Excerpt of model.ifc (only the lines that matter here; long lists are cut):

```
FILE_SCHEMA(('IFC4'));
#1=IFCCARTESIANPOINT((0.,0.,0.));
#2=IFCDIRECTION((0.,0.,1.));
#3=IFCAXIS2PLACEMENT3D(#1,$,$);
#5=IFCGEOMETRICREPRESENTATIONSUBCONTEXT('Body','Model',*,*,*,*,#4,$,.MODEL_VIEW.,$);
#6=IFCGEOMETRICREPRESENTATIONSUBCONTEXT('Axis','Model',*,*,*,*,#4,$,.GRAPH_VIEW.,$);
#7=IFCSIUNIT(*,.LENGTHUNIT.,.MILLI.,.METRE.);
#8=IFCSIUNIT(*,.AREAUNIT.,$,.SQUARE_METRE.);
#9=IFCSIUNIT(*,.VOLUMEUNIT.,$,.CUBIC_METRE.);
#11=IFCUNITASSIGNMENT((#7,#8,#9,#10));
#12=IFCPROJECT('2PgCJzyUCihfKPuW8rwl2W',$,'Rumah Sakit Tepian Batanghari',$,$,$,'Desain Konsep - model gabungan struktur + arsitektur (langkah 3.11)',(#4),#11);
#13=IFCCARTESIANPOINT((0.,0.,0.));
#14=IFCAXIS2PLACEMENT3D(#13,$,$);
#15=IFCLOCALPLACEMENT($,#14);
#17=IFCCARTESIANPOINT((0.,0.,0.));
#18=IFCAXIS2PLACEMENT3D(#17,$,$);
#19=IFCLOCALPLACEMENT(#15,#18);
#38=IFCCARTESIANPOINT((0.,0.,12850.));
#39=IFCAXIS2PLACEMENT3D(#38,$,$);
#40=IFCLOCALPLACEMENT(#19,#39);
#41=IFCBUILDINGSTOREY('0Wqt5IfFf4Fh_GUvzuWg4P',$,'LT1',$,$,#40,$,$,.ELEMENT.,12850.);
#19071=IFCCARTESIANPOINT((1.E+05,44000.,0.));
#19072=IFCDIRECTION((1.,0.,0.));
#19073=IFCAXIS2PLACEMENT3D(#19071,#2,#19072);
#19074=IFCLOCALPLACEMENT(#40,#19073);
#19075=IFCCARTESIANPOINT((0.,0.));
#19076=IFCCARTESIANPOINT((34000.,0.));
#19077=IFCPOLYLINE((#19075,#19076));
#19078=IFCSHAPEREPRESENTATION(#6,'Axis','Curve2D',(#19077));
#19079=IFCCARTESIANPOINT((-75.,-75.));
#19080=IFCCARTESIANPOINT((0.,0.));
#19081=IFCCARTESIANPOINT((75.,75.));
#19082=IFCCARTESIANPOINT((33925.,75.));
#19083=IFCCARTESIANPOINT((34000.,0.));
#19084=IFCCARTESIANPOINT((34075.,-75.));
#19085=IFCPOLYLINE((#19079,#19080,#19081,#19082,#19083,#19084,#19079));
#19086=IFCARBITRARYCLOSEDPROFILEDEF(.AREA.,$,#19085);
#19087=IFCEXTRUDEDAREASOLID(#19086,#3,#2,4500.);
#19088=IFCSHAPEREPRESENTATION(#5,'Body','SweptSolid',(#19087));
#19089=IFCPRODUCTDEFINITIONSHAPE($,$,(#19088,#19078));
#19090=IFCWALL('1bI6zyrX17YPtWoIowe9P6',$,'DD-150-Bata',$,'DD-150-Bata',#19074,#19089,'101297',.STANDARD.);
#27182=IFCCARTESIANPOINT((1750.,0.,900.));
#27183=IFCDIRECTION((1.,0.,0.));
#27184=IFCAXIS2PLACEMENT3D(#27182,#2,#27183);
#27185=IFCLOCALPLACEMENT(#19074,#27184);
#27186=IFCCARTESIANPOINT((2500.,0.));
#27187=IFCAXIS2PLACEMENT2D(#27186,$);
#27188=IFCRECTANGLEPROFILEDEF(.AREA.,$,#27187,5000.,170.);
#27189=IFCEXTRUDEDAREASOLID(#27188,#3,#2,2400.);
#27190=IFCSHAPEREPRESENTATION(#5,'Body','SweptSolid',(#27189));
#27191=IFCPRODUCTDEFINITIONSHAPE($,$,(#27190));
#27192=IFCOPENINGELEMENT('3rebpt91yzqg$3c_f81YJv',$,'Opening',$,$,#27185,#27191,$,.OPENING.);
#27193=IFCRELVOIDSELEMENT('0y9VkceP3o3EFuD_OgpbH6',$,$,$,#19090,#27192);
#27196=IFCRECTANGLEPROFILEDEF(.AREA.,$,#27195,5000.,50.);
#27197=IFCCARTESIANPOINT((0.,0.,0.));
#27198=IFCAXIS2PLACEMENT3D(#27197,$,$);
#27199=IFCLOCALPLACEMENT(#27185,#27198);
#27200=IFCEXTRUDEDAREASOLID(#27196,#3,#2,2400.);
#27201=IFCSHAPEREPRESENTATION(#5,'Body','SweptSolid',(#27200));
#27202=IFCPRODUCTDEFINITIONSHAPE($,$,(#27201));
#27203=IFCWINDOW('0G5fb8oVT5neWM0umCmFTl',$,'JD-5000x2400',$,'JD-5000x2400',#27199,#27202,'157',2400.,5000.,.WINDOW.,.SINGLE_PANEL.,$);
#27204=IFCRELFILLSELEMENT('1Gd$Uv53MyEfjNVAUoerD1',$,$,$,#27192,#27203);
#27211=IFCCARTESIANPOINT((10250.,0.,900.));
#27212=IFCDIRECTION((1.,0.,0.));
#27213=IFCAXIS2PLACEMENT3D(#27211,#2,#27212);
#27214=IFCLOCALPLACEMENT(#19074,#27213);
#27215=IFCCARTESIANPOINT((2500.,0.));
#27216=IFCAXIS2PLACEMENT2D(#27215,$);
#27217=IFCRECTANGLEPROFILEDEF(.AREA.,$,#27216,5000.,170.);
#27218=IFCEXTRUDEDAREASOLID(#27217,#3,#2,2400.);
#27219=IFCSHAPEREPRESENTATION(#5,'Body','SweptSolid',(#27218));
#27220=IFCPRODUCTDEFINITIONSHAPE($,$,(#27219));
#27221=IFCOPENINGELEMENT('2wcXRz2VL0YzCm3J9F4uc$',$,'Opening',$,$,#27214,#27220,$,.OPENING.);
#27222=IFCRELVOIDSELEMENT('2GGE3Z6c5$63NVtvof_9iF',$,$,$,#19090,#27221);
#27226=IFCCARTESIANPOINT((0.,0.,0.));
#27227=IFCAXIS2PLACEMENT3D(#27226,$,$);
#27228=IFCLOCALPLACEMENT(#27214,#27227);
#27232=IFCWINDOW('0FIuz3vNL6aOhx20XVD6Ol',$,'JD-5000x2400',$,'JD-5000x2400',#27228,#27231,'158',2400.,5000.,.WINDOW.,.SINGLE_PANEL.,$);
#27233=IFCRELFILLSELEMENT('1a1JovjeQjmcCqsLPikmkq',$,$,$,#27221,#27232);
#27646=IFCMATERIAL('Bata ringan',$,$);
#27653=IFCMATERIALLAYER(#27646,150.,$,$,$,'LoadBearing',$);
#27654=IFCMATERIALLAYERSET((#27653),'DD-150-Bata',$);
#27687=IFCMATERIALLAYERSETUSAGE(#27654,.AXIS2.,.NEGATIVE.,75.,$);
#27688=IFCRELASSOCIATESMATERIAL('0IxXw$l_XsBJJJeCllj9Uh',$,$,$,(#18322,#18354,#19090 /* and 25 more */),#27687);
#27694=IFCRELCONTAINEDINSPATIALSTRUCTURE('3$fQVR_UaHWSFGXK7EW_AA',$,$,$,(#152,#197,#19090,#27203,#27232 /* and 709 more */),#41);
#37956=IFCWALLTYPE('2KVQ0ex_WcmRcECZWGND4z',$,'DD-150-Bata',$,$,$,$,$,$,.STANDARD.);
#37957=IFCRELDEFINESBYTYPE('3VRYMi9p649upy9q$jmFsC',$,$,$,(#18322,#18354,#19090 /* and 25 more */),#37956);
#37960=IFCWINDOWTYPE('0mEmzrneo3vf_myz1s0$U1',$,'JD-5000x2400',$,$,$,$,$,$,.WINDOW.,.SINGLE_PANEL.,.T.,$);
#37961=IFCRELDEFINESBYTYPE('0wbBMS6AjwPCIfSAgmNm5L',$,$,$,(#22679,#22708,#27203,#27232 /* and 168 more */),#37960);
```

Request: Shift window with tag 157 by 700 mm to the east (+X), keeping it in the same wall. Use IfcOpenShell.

```python
import ifcopenshell
import ifcopenshell.api.geometry
import ifcopenshell.util.placement
import ifcopenshell.util.unit

model = ifcopenshell.open("model.ifc")
unit_scale = ifcopenshell.util.unit.calculate_unit_scale(model)

window = model.by_guid("0G5fb8oVT5neWM0umCmFTl")
opening = window.FillsVoids[0].RelatingOpeningElement
wall = opening.VoidsElements[0].RelatingBuildingElement

wall_matrix = ifcopenshell.util.placement.get_local_placement(wall.ObjectPlacement)
shift = wall_matrix[:3, 0] * 0.7 / unit_scale
before = ifcopenshell.util.placement.get_local_placement(window.ObjectPlacement)[:3, 3].copy()

# The window is placed relative to its opening, so it follows when the opening moves.
matrix = ifcopenshell.util.placement.get_local_placement(opening.ObjectPlacement)
matrix[:3, 3] += shift
ifcopenshell.api.geometry.edit_object_placement(
    model, product=opening, matrix=matrix, is_si=False, should_transform_children=True
)

after = ifcopenshell.util.placement.get_local_placement(window.ObjectPlacement)[:3, 3]
print("window moved by", (after - before).round(3) + 0.0)

model.write("model_rev.ifc")
```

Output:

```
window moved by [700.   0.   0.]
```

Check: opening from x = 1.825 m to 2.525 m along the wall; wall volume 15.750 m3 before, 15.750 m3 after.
